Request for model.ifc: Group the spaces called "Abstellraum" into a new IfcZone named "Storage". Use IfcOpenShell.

First a look at what the model holds.

```python
import ifcopenshell

model = ifcopenshell.open("model.ifc")
print(model.schema)
seen = {}
for space in model.by_type("IfcSpace"):
    seen[space.LongName] = seen.get(space.LongName, 0) + 1
for name, count in sorted(seen.items(), key=str):
    print(count, "x", name)
print("zones:", [z.Name for z in model.by_type("IfcZone")][:20])
```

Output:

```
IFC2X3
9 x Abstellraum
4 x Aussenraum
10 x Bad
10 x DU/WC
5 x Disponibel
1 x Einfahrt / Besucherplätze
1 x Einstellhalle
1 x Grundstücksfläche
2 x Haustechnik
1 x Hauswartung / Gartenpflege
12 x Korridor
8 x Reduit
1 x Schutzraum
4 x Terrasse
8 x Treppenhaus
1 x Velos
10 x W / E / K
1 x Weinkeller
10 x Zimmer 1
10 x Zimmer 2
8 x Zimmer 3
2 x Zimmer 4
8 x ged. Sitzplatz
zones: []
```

```python
import ifcopenshell
import ifcopenshell.api.group
import ifcopenshell.api.root

model = ifcopenshell.open("model.ifc")

names = {"Abstellraum"}
spaces = [s for s in model.by_type("IfcSpace") if s.LongName in names]

zone = ifcopenshell.api.root.create_entity(model, ifc_class="IfcZone", name="Storage")
ifcopenshell.api.group.assign_group(model, products=spaces, group=zone)
print(len(spaces), "spaces in", zone.Name)

model.write("model_edited.ifc")
```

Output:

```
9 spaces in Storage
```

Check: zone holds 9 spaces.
